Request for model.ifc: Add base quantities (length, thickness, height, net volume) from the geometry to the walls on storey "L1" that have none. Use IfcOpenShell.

First a look at what the model holds.

```python
import ifcopenshell
import ifcopenshell.util.element
import ifcopenshell.util.unit

model = ifcopenshell.open("model.ifc")
print(model.schema)
for unit_type in ("LENGTHUNIT", "AREAUNIT", "VOLUMEUNIT"):
    print(unit_type, ifcopenshell.util.unit.calculate_unit_scale(model, unit_type))
storey = next(s for s in model.by_type("IfcBuildingStorey") if s.Name == "L1")
walls = [e for e in ifcopenshell.util.element.get_decomposition(storey) if e.is_a("IfcWall")]
for e in sorted(walls, key=lambda e: e.id()):
    print(e.id(), e.is_a(), e.Name, list(ifcopenshell.util.element.get_psets(e, qtos_only=True)), sep=" | ")
```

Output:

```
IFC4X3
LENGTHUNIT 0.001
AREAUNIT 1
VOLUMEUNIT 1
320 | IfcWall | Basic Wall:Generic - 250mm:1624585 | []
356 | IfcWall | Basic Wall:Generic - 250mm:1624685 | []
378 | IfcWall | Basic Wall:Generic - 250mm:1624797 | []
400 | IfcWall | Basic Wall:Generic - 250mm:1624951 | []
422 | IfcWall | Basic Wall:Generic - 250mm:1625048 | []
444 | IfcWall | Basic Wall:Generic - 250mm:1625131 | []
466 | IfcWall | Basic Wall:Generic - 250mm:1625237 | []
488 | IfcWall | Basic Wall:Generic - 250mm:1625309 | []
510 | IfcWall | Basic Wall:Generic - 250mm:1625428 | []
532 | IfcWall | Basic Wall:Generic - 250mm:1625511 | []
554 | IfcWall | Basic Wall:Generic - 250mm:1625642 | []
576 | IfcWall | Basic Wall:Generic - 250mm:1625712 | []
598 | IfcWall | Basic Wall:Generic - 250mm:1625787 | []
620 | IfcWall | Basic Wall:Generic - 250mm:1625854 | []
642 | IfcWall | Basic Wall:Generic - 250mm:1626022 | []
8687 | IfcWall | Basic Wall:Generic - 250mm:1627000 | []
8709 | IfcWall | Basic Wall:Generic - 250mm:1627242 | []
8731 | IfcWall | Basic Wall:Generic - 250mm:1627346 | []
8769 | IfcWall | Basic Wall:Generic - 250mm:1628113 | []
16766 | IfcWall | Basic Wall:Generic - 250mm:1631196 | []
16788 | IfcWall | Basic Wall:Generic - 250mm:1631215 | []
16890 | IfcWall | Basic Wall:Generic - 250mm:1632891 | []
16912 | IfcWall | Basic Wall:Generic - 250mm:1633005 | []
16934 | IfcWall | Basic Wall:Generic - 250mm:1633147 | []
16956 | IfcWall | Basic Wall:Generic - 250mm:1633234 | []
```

```python
import ifcopenshell
import ifcopenshell.api.pset
import ifcopenshell.geom
import ifcopenshell.util.element
import ifcopenshell.util.shape
import ifcopenshell.util.unit

model = ifcopenshell.open("model.ifc")
unit_scale = ifcopenshell.util.unit.calculate_unit_scale(model)
volume_scale = ifcopenshell.util.unit.calculate_unit_scale(model, "VOLUMEUNIT")
settings = ifcopenshell.geom.settings()

storey = next(s for s in model.by_type("IfcBuildingStorey") if s.Name == "L1")
walls = [e for e in ifcopenshell.util.element.get_decomposition(storey) if e.is_a("IfcWall")]

for e in sorted(walls, key=lambda e: e.id()):
    if ifcopenshell.util.element.get_psets(e, qtos_only=True, should_inherit=False):
        continue
    # Geometry comes back in metres, in the element's own axes.
    shape = ifcopenshell.geom.create_shape(settings, e)
    values = {
        "Length": ifcopenshell.util.shape.get_x(shape.geometry) / unit_scale,
        "Width": ifcopenshell.util.shape.get_y(shape.geometry) / unit_scale,
        "Height": ifcopenshell.util.shape.get_z(shape.geometry) / unit_scale,
        "NetVolume": ifcopenshell.util.shape.get_volume(shape.geometry) / volume_scale,
    }
    qto = ifcopenshell.api.pset.add_qto(model, product=e, name="Qto_WallBaseQuantities")
    ifcopenshell.api.pset.edit_qto(model, qto=qto, properties=values)
    print(e.id(), {k: round(v, 3) for k, v in values.items()})

model.write("model_rev.ifc")
```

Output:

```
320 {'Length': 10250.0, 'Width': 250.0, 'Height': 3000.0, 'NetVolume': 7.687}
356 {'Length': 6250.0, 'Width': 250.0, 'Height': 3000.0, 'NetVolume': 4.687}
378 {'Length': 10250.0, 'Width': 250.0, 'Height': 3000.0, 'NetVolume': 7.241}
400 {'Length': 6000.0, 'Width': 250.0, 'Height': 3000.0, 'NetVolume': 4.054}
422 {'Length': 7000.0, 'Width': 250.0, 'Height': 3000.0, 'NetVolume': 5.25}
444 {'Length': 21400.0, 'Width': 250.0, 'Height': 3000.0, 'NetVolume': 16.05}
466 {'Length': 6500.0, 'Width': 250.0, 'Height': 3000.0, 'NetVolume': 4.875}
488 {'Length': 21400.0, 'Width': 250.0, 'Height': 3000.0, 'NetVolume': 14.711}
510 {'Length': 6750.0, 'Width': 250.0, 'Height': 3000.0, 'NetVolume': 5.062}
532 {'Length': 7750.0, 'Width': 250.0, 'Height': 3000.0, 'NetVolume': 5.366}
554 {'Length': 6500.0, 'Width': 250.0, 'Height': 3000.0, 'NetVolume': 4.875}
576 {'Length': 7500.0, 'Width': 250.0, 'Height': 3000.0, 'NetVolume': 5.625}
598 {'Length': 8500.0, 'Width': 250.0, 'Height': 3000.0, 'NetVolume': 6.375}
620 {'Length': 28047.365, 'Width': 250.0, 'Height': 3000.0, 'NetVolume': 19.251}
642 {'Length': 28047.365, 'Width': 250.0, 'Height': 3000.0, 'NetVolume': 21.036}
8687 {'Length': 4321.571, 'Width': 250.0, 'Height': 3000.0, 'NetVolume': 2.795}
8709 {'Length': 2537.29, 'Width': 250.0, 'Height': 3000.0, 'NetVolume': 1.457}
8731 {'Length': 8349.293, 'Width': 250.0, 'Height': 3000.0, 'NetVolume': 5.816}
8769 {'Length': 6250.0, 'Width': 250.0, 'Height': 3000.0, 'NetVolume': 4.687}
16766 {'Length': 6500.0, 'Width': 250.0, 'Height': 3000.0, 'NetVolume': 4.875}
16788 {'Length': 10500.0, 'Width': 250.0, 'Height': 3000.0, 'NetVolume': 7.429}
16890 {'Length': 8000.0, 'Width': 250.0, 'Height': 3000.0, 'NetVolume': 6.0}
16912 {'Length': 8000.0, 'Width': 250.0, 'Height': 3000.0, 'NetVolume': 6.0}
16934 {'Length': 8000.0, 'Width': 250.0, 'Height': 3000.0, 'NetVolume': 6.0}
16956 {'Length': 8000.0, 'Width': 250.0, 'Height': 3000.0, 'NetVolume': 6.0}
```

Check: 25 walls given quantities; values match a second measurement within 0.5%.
